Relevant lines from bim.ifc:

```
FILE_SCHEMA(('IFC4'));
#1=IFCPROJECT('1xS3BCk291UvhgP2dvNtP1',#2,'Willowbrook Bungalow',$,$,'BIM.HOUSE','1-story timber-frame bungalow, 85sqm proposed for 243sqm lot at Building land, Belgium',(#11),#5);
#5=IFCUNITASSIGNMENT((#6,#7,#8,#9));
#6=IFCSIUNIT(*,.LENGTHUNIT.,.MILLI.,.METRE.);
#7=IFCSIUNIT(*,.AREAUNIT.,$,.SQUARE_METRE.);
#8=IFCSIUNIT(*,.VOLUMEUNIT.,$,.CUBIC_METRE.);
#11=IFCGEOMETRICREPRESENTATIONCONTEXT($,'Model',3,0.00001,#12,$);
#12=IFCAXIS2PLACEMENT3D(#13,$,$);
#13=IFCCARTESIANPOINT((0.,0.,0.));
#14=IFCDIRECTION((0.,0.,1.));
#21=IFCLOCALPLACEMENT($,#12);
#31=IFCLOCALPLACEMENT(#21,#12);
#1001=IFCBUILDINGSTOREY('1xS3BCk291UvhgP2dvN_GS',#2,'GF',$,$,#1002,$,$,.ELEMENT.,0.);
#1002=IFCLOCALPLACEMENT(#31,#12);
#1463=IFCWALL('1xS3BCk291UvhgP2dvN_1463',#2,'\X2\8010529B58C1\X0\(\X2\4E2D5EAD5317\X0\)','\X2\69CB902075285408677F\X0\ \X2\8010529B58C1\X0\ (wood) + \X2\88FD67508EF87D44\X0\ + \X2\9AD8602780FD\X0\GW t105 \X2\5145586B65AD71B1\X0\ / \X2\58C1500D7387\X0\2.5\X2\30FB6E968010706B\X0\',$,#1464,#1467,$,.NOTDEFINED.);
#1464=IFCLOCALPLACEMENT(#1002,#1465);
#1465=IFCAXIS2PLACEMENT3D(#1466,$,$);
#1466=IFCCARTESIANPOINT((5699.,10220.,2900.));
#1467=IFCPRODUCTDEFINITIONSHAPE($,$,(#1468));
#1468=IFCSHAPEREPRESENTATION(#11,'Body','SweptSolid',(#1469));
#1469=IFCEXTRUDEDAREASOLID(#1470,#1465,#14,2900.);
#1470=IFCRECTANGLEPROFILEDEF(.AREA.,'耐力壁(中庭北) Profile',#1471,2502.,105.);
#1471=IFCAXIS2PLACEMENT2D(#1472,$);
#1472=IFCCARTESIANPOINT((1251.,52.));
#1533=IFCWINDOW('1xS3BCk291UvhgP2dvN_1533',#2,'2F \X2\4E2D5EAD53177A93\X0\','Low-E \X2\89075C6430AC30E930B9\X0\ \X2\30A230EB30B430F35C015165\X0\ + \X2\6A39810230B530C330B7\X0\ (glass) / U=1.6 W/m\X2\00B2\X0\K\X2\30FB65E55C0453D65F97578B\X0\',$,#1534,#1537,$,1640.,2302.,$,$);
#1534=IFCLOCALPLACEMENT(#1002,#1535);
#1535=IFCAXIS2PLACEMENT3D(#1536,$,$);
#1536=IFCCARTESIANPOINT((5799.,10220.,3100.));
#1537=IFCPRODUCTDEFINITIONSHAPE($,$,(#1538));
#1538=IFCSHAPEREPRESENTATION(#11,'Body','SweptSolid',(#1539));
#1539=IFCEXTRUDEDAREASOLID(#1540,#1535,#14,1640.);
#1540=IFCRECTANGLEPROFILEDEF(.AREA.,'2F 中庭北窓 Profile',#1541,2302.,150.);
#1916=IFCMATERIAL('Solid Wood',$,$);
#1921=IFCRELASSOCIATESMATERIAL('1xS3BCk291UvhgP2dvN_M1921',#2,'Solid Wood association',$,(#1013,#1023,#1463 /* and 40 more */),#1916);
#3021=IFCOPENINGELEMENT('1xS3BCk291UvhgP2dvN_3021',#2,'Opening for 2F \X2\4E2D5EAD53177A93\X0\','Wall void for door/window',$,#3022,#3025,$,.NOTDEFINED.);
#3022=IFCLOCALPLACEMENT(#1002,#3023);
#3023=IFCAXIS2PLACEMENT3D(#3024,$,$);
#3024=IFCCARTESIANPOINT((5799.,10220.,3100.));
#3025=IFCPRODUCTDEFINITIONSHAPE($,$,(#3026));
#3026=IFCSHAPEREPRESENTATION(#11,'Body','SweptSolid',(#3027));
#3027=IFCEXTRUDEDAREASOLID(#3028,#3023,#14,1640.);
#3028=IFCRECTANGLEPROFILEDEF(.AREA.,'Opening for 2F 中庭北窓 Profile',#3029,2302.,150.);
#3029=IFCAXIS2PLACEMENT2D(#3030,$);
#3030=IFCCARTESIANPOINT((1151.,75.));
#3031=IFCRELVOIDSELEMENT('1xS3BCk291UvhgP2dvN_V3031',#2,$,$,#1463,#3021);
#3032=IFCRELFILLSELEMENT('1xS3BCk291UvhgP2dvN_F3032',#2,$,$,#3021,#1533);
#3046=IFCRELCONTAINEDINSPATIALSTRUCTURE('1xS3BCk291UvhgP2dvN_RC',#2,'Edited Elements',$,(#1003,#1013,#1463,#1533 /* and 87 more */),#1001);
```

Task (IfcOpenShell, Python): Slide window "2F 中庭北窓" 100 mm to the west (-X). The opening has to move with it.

```python
import ifcopenshell
import ifcopenshell.api.geometry
import ifcopenshell.util.placement
import ifcopenshell.util.unit

model = ifcopenshell.open("bim.ifc")
unit_scale = ifcopenshell.util.unit.calculate_unit_scale(model)

window = model.by_guid("1xS3BCk291UvhgP2dvN_1533")
opening = window.FillsVoids[0].RelatingOpeningElement
wall = opening.VoidsElements[0].RelatingBuildingElement

wall_matrix = ifcopenshell.util.placement.get_local_placement(wall.ObjectPlacement)
shift = wall_matrix[:3, 0] * -0.1 / unit_scale
before = ifcopenshell.util.placement.get_local_placement(window.ObjectPlacement)[:3, 3].copy()

# The window is not placed relative to its opening, so move both.
for product in (opening, window):
    matrix = ifcopenshell.util.placement.get_local_placement(product.ObjectPlacement)
    matrix[:3, 3] += shift
    ifcopenshell.api.geometry.edit_object_placement(model, product=product, matrix=matrix, is_si=False)

after = ifcopenshell.util.placement.get_local_placement(window.ObjectPlacement)[:3, 3]
print("window moved by", (after - before).round(3) + 0.0)

model.write("bim-out.ifc")
```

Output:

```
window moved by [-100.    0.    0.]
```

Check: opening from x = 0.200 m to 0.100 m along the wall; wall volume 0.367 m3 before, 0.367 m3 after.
